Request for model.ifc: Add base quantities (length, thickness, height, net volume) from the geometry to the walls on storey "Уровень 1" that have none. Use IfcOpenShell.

First a look at what the model holds.

```python
import ifcopenshell
import ifcopenshell.util.element
import ifcopenshell.util.unit

model = ifcopenshell.open("model.ifc")
print(model.schema)
for unit_type in ("LENGTHUNIT", "AREAUNIT", "VOLUMEUNIT"):
    print(unit_type, ifcopenshell.util.unit.calculate_unit_scale(model, unit_type))
storey = next(s for s in model.by_type("IfcBuildingStorey") if s.Name == "Уровень 1")
walls = [e for e in ifcopenshell.util.element.get_decomposition(storey) if e.is_a("IfcWall")]
for e in sorted(walls, key=lambda e: e.id()):
    print(e.id(), e.is_a(), e.Name, list(ifcopenshell.util.element.get_psets(e, qtos_only=True)), sep=" | ")
```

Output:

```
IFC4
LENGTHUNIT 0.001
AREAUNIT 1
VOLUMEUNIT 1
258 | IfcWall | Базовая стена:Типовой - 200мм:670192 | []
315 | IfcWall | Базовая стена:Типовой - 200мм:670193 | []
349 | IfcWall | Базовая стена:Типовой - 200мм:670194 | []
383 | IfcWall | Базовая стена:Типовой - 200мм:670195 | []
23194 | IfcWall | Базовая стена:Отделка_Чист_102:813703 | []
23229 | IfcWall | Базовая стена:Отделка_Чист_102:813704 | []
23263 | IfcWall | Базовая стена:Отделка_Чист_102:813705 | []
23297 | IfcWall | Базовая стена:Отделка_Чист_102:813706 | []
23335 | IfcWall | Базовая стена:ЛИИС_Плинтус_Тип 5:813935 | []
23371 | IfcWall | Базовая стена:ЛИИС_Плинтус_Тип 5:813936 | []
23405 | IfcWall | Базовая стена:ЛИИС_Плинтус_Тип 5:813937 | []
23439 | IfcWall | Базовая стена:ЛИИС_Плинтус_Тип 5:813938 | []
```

```python
import ifcopenshell
import ifcopenshell.api.pset
import ifcopenshell.geom
import ifcopenshell.util.element
import ifcopenshell.util.shape
import ifcopenshell.util.unit

model = ifcopenshell.open("model.ifc")
unit_scale = ifcopenshell.util.unit.calculate_unit_scale(model)
volume_scale = ifcopenshell.util.unit.calculate_unit_scale(model, "VOLUMEUNIT")
settings = ifcopenshell.geom.settings()

storey = next(s for s in model.by_type("IfcBuildingStorey") if s.Name == "Уровень 1")
walls = [e for e in ifcopenshell.util.element.get_decomposition(storey) if e.is_a("IfcWall")]

for e in sorted(walls, key=lambda e: e.id()):
    if ifcopenshell.util.element.get_psets(e, qtos_only=True, should_inherit=False):
        continue
    # Geometry comes back in metres, in the element's own axes.
    shape = ifcopenshell.geom.create_shape(settings, e)
    values = {
        "Length": ifcopenshell.util.shape.get_x(shape.geometry) / unit_scale,
        "Width": ifcopenshell.util.shape.get_y(shape.geometry) / unit_scale,
        "Height": ifcopenshell.util.shape.get_z(shape.geometry) / unit_scale,
        "NetVolume": ifcopenshell.util.shape.get_volume(shape.geometry) / volume_scale,
    }
    qto = ifcopenshell.api.pset.add_qto(model, product=e, name="Qto_WallBaseQuantities")
    ifcopenshell.api.pset.edit_qto(model, qto=qto, properties=values)
    print(e.id(), {k: round(v, 3) for k, v in values.items()})

model.write("model_updated.ifc")
```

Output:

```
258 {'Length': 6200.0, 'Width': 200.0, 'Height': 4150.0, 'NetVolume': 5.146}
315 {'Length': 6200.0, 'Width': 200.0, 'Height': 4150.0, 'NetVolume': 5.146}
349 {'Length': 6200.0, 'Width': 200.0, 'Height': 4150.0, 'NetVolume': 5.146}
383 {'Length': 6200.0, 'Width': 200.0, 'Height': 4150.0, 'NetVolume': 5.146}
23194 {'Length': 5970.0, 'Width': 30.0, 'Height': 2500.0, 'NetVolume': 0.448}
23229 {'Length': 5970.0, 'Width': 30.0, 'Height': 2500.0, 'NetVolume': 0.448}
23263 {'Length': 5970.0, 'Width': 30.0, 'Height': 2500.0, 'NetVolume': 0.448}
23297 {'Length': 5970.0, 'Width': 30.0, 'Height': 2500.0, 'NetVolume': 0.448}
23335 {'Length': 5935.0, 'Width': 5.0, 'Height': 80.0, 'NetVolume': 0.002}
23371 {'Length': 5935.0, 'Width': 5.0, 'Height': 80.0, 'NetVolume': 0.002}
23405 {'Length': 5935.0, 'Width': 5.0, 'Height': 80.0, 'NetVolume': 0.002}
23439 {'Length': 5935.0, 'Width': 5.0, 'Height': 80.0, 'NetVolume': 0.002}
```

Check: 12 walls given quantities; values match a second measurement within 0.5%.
